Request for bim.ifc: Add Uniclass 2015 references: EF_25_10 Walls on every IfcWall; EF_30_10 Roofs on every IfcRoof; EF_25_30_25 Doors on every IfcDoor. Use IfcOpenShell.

First a look at what the model holds.

```python
import ifcopenshell

model = ifcopenshell.open("bim.ifc")
print(model.schema)
print("classifications:", [c.Name for c in model.by_type("IfcClassification")])
for ifc_class in ("IfcDoor", "IfcRoof", "IfcStair", "IfcWall", "IfcWindow"):
    print(ifc_class, len(model.by_type(ifc_class)))
```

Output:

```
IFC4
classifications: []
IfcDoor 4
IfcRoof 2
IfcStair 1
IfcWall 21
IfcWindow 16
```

```python
import ifcopenshell
import ifcopenshell.api.classification

model = ifcopenshell.open("bim.ifc")

system = ifcopenshell.api.classification.add_classification(model, classification="Uniclass 2015")

codes = {
    "IfcWall": ("EF_25_10", "Walls"),
    "IfcRoof": ("EF_30_10", "Roofs"),
    "IfcDoor": ("EF_25_30_25", "Doors"),
}
for ifc_class, (code, name) in codes.items():
    products = model.by_type(ifc_class)
    ifcopenshell.api.classification.add_reference(
        model, products=products, classification=system, identification=code, name=name
    )
    print(code, len(products))

model.write("bim_rev.ifc")
```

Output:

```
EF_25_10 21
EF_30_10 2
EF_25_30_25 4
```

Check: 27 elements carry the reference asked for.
